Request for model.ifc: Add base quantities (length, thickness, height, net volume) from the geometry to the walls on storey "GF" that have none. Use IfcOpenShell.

First a look at what the model holds.

```python
import ifcopenshell
import ifcopenshell.util.element
import ifcopenshell.util.unit

model = ifcopenshell.open("model.ifc")
print(model.schema)
for unit_type in ("LENGTHUNIT", "AREAUNIT", "VOLUMEUNIT"):
    print(unit_type, ifcopenshell.util.unit.calculate_unit_scale(model, unit_type))
storey = next(s for s in model.by_type("IfcBuildingStorey") if s.Name == "GF")
walls = [e for e in ifcopenshell.util.element.get_decomposition(storey) if e.is_a("IfcWall")]
for e in sorted(walls, key=lambda e: e.id()):
    print(e.id(), e.is_a(), e.Name, list(ifcopenshell.util.element.get_psets(e, qtos_only=True)), sep=" | ")
```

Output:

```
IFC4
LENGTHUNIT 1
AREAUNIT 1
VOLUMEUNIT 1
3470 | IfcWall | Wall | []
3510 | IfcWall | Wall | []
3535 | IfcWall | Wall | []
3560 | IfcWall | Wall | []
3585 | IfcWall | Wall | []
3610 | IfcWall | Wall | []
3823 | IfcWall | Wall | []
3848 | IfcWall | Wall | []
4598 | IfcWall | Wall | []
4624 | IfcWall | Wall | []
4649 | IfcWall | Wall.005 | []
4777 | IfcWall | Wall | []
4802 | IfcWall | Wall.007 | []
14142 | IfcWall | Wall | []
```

```python
import ifcopenshell
import ifcopenshell.api.pset
import ifcopenshell.geom
import ifcopenshell.util.element
import ifcopenshell.util.shape
import ifcopenshell.util.unit

model = ifcopenshell.open("model.ifc")
unit_scale = ifcopenshell.util.unit.calculate_unit_scale(model)
volume_scale = ifcopenshell.util.unit.calculate_unit_scale(model, "VOLUMEUNIT")
settings = ifcopenshell.geom.settings()

storey = next(s for s in model.by_type("IfcBuildingStorey") if s.Name == "GF")
walls = [e for e in ifcopenshell.util.element.get_decomposition(storey) if e.is_a("IfcWall")]

for e in sorted(walls, key=lambda e: e.id()):
    if ifcopenshell.util.element.get_psets(e, qtos_only=True, should_inherit=False):
        continue
    # Geometry comes back in metres, in the element's own axes.
    shape = ifcopenshell.geom.create_shape(settings, e)
    values = {
        "Length": ifcopenshell.util.shape.get_x(shape.geometry) / unit_scale,
        "Width": ifcopenshell.util.shape.get_y(shape.geometry) / unit_scale,
        "Height": ifcopenshell.util.shape.get_z(shape.geometry) / unit_scale,
        "NetVolume": ifcopenshell.util.shape.get_volume(shape.geometry) / volume_scale,
    }
    qto = ifcopenshell.api.pset.add_qto(model, product=e, name="Qto_WallBaseQuantities")
    ifcopenshell.api.pset.edit_qto(model, qto=qto, properties=values)
    print(e.id(), {k: round(v, 3) for k, v in values.items()})

model.write("model_rev.ifc")
```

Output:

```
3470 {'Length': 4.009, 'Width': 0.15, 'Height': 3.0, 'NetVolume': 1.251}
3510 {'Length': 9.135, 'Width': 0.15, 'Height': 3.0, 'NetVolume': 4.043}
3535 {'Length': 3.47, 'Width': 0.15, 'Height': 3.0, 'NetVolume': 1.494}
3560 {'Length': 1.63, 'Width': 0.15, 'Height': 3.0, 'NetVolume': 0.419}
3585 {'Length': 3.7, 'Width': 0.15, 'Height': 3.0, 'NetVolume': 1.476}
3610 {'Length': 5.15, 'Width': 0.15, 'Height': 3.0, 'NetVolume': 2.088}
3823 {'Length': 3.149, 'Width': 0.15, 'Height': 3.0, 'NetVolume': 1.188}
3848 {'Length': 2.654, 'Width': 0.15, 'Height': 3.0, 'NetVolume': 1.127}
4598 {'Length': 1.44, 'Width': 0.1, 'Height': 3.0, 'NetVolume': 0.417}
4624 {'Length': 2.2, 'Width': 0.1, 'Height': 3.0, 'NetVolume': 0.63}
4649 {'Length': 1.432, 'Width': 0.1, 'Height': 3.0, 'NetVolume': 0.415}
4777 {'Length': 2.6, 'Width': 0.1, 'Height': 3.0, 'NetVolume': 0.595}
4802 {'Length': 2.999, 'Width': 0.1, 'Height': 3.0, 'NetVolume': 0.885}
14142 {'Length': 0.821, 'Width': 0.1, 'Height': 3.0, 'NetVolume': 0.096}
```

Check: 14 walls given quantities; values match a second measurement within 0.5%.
